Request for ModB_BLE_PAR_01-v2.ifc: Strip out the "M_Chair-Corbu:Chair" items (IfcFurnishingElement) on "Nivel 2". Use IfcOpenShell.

First a look at what the model holds.

```python
import ifcopenshell
import ifcopenshell.util.element

model = ifcopenshell.open("ModB_BLE_PAR_01-v2.ifc")
print(model.schema)
storey = next(s for s in model.by_type("IfcBuildingStorey") if s.Name == "Nivel 2")
furniture = [e for e in ifcopenshell.util.element.get_decomposition(storey) if e.is_a("IfcFurnishingElement")]
seen = {}
for e in furniture:
    element_type = ifcopenshell.util.element.get_type(e)
    name = element_type.Name if element_type not in (None, e) else None
    seen[name] = seen.get(name, 0) + 1
for name, count in sorted(seen.items(), key=str):
    print(count, "x", name)
```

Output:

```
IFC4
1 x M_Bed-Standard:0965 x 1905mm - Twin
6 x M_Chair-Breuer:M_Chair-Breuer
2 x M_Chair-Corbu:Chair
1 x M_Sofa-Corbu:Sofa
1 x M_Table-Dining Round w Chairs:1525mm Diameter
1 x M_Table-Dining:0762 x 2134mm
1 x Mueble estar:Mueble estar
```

```python
import ifcopenshell
import ifcopenshell.api.root
import ifcopenshell.util.element

model = ifcopenshell.open("ModB_BLE_PAR_01-v2.ifc")

storey = next(s for s in model.by_type("IfcBuildingStorey") if s.Name == "Nivel 2")
furniture = [e for e in ifcopenshell.util.element.get_decomposition(storey) if e.is_a("IfcFurnishingElement")]
targets = [e for e in furniture if (t := ifcopenshell.util.element.get_type(e)) not in (None, e) and t.Name == "M_Chair-Corbu:Chair"]

for e in targets:
    ifcopenshell.api.root.remove_product(model, product=e)
print(len(targets), "removed")

model.write("ModB_BLE_PAR_01-v2_updated.ifc")
```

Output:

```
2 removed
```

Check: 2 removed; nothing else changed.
